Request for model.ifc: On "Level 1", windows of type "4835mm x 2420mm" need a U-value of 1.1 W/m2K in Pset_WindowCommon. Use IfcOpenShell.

First a look at what the model holds.

```python
import ifcopenshell
import ifcopenshell.util.element

model = ifcopenshell.open("model.ifc")
print(model.schema)
storey = next(s for s in model.by_type("IfcBuildingStorey") if s.Name == "Level 1")
windows = [e for e in ifcopenshell.util.element.get_decomposition(storey) if e.is_a("IfcWindow")]
seen = {}
for e in windows:
    element_type = ifcopenshell.util.element.get_type(e)
    key = (element_type.Name if element_type != e and element_type else None, ifcopenshell.util.element.get_pset(e, "Pset_WindowCommon", "ThermalTransmittance"))
    seen[key] = seen.get(key, 0) + 1
for (name, value), count in sorted(seen.items(), key=str):
    print(count, "x", name, "|", value)
```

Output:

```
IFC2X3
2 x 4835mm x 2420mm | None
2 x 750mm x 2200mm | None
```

```python
import ifcopenshell
import ifcopenshell.api.pset
import ifcopenshell.util.element

model = ifcopenshell.open("model.ifc")

storey = next(s for s in model.by_type("IfcBuildingStorey") if s.Name == "Level 1")
windows = [e for e in ifcopenshell.util.element.get_decomposition(storey) if e.is_a("IfcWindow")]

count = 0
for e in windows:
    element_type = ifcopenshell.util.element.get_type(e)
    if element_type in (None, e) or element_type.Name != "4835mm x 2420mm":
        continue
    # add_pset returns the element's existing set when there is one.
    pset = ifcopenshell.api.pset.add_pset(model, product=e, name="Pset_WindowCommon")
    ifcopenshell.api.pset.edit_pset(model, pset=pset, properties={"ThermalTransmittance": 1.1})
    count += 1

print(count, "windows updated")

model.write("model-out.ifc")
```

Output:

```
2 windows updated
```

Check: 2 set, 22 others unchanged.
